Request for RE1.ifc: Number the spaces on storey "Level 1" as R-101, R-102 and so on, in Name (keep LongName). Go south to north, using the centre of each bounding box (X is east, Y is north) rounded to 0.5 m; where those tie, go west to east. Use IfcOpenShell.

First a look at what the model holds.

```python
import ifcopenshell
import ifcopenshell.util.element
import ifcopenshell.util.placement

model = ifcopenshell.open("RE1.ifc")
print(model.schema)
storey = next(s for s in model.by_type("IfcBuildingStorey") if s.Name == "Level 1")
spaces = [e for e in ifcopenshell.util.element.get_decomposition(storey) if e.is_a("IfcSpace")]
for e in sorted(spaces, key=lambda e: e.id()):
    origin = ifcopenshell.util.placement.get_local_placement(e.ObjectPlacement)[:3, 3]
    print(e.id(), e.Name, e.LongName, origin.round(2) + 0.0, sep=" | ")
```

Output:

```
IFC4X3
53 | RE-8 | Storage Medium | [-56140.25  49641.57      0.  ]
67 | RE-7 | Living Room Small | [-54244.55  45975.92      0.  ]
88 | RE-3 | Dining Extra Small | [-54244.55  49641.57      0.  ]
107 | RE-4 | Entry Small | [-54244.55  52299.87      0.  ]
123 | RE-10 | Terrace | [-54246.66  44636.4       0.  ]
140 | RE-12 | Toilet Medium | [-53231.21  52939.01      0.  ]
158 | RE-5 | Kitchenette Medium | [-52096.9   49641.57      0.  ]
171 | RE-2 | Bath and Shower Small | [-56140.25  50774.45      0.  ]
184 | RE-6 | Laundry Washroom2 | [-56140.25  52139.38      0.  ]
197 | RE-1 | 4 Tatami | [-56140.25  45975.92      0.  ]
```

```python
import ifcopenshell
import ifcopenshell.geom
import ifcopenshell.util.element
import ifcopenshell.util.shape

model = ifcopenshell.open("RE1.ifc")
settings = ifcopenshell.geom.settings()
settings.set("use-world-coords", True)


def centre(element):
    shape = ifcopenshell.geom.create_shape(settings, element)
    return ifcopenshell.util.shape.get_bbox_centroid(shape.geometry)


storey = next(s for s in model.by_type("IfcBuildingStorey") if s.Name == "Level 1")
spaces = [e for e in ifcopenshell.util.element.get_decomposition(storey) if e.is_a("IfcSpace")]

# Insertion points can sit at a corner or the storey origin, so sort by the geometry (in metres).
centres = {e: centre(e) for e in spaces}
spaces.sort(key=lambda e: (round(centres[e][1] / 0.5), centres[e][0]))

for i, e in enumerate(spaces, start=1):
    number = f"R-1{i:02d}"
    e.Name = number
    print(e.id(), number)

model.write("RE1_edited.ifc")
```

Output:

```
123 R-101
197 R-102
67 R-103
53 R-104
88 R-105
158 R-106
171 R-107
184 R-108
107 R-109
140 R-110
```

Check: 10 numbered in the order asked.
